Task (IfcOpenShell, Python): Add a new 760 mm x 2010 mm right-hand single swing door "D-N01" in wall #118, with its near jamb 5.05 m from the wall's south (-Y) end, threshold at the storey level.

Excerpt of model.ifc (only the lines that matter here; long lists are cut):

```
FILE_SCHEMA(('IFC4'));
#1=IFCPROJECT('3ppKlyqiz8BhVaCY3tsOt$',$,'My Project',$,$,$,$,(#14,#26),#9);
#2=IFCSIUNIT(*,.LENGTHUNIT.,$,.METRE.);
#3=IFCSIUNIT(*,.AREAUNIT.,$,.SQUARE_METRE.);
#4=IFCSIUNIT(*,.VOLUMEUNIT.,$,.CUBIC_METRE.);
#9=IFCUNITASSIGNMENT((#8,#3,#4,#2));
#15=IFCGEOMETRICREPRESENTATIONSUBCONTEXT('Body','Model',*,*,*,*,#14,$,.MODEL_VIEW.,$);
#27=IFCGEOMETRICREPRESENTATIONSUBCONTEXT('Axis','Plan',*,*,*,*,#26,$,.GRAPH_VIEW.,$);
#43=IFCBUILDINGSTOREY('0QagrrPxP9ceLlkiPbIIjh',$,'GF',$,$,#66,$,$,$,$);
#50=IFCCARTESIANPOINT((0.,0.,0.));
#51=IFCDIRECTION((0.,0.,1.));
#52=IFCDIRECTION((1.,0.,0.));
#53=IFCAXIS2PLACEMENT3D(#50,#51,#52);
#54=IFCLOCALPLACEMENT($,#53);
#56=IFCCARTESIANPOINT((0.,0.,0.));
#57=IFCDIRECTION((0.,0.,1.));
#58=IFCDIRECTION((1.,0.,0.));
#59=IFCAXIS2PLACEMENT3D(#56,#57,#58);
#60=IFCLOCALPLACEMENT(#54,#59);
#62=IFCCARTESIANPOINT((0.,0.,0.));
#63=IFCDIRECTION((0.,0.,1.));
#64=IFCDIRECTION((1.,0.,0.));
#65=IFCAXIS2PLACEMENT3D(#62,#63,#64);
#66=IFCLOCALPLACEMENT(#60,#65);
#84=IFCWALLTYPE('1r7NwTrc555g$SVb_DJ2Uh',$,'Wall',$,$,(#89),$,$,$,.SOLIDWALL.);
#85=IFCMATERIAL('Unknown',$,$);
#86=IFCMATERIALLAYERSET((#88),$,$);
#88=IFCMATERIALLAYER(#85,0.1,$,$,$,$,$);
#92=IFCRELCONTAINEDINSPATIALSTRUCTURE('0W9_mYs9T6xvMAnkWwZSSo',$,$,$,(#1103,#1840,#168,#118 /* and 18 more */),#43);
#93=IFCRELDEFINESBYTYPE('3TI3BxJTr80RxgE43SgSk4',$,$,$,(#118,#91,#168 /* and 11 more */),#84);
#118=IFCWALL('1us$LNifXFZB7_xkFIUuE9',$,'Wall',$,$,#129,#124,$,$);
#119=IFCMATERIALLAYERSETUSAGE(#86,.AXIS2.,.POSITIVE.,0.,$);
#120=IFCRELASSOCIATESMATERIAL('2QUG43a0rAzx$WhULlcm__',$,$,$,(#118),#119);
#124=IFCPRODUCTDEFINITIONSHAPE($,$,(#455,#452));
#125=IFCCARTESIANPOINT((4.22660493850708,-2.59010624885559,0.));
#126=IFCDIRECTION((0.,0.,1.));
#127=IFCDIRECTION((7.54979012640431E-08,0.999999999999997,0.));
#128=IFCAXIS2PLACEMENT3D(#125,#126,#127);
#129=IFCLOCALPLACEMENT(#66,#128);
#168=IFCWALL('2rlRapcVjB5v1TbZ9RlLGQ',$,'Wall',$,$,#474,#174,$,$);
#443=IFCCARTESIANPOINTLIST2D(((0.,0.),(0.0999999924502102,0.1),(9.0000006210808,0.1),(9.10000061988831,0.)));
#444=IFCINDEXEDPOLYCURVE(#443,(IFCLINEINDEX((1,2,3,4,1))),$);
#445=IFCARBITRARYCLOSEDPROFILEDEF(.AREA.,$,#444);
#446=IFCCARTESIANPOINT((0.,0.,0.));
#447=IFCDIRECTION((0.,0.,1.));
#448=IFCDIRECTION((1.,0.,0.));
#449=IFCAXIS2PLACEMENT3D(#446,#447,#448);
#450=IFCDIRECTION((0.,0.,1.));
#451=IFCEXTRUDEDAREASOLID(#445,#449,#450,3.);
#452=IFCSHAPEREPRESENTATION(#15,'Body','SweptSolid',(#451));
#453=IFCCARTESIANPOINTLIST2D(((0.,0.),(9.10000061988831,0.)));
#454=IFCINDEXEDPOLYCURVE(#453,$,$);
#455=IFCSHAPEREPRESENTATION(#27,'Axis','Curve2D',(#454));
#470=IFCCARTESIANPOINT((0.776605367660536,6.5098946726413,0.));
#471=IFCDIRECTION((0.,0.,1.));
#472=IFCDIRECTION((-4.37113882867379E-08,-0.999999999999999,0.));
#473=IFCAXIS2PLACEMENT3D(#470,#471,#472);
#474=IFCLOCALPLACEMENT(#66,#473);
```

```python
import numpy as np
import ifcopenshell
import ifcopenshell.api.feature
import ifcopenshell.api.geometry
import ifcopenshell.api.root
import ifcopenshell.api.spatial
import ifcopenshell.geom
import ifcopenshell.util.element
import ifcopenshell.util.placement
import ifcopenshell.util.representation
import ifcopenshell.util.shape
import ifcopenshell.util.unit

model = ifcopenshell.open("model.ifc")
unit_scale = ifcopenshell.util.unit.calculate_unit_scale(model)
settings = ifcopenshell.geom.settings()


def volume(element):
    """Net volume in cubic metres, openings subtracted."""
    shape = ifcopenshell.geom.create_shape(settings, element)
    return ifcopenshell.util.shape.get_volume(shape.geometry)


wall = model.by_id(118)
storey = ifcopenshell.util.element.get_container(wall, ifc_class="IfcBuildingStorey")
context = ifcopenshell.util.representation.get_context(model, "Model", "Body", "MODEL_VIEW")
before = volume(wall)

width, height, from_end, sill = 0.76, 2.01, 5.05, 0.0  # metres

# The wall runs along its own X axis, and the end named is its -X end.
wall_shape = ifcopenshell.geom.create_shape(settings, wall)
x, y, z = ifcopenshell.util.shape.get_vertices(wall_shape.geometry).T
start = x.min() + from_end
face, thickness = float(y.min()), float(y.max() - y.min())
wall_matrix = ifcopenshell.util.placement.get_local_placement(wall.ObjectPlacement)
level = ifcopenshell.util.placement.get_local_placement(storey.ObjectPlacement)[2, 3]


def in_wall(x, y):
    """Placement at x, y metres in the wall's axes, at sill height."""
    matrix = wall_matrix.copy()
    matrix[:, 3] = wall_matrix @ np.array([x / unit_scale, y / unit_scale, 0.0, 1.0])
    matrix[2, 3] = level + sill / unit_scale
    return matrix


# Opening: a box that overshoots both wall faces by 50 mm.
opening = ifcopenshell.api.root.create_entity(model, ifc_class="IfcOpeningElement", predefined_type="OPENING")
box = ifcopenshell.api.geometry.add_wall_representation(
    model, context=context, length=width, height=height, thickness=thickness + 0.1
)
ifcopenshell.api.geometry.assign_representation(model, product=opening, representation=box)
ifcopenshell.api.geometry.edit_object_placement(model, product=opening, matrix=in_wall(start, face - 0.05), is_si=False)
ifcopenshell.api.feature.add_feature(model, feature=opening, element=wall)

door = ifcopenshell.api.root.create_entity(model, ifc_class="IfcDoor", name="D-N01", predefined_type="DOOR")
door.OverallWidth, door.OverallHeight = width / unit_scale, height / unit_scale
door.OperationType = "SINGLE_SWING_RIGHT"
body = ifcopenshell.api.geometry.add_door_representation(
    model,
    context=context,
    overall_width=door.OverallWidth,
    overall_height=door.OverallHeight,
    operation_type="SINGLE_SWING_RIGHT",
    lining_properties={"LiningDepth": thickness / unit_scale, "ThresholdDepth": thickness / unit_scale},
)
ifcopenshell.api.geometry.assign_representation(model, product=door, representation=body)
ifcopenshell.api.spatial.assign_container(model, products=[door], relating_structure=storey)
ifcopenshell.api.feature.add_filling(model, opening=opening, element=door)

# The lining spans the wall, so the door starts at the wall face.
ifcopenshell.api.geometry.edit_object_placement(model, product=door, matrix=in_wall(start, face), is_si=False)

after = volume(wall)

print(f"wall volume {before:.3f} -> {after:.3f} m3")

model.write("model-out.ifc")
```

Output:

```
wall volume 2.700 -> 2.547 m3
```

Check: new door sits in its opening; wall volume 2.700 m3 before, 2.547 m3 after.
